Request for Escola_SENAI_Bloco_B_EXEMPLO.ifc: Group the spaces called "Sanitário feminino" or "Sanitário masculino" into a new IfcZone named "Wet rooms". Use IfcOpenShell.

First a look at what the model holds.

```python
import ifcopenshell

model = ifcopenshell.open("Escola_SENAI_Bloco_B_EXEMPLO.ifc")
print(model.schema)
seen = {}
for space in model.by_type("IfcSpace"):
    seen[space.LongName] = seen.get(space.LongName, 0) + 1
for name, count in sorted(seen.items(), key=str):
    print(count, "x", name)
print("zones:", [z.Name for z in model.by_type("IfcZone")][:20])
```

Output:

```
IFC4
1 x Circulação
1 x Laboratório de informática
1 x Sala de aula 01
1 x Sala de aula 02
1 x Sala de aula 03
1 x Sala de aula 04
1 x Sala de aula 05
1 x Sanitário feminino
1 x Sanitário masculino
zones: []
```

```python
import ifcopenshell
import ifcopenshell.api.group
import ifcopenshell.api.root

model = ifcopenshell.open("Escola_SENAI_Bloco_B_EXEMPLO.ifc")

names = {"Sanitário feminino", "Sanitário masculino"}
spaces = [s for s in model.by_type("IfcSpace") if s.LongName in names]

zone = ifcopenshell.api.root.create_entity(model, ifc_class="IfcZone", name="Wet rooms")
ifcopenshell.api.group.assign_group(model, products=spaces, group=zone)
print(len(spaces), "spaces in", zone.Name)

model.write("Escola_SENAI_Bloco_B_EXEMPLO-out.ifc")
```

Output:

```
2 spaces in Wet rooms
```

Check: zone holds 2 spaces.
